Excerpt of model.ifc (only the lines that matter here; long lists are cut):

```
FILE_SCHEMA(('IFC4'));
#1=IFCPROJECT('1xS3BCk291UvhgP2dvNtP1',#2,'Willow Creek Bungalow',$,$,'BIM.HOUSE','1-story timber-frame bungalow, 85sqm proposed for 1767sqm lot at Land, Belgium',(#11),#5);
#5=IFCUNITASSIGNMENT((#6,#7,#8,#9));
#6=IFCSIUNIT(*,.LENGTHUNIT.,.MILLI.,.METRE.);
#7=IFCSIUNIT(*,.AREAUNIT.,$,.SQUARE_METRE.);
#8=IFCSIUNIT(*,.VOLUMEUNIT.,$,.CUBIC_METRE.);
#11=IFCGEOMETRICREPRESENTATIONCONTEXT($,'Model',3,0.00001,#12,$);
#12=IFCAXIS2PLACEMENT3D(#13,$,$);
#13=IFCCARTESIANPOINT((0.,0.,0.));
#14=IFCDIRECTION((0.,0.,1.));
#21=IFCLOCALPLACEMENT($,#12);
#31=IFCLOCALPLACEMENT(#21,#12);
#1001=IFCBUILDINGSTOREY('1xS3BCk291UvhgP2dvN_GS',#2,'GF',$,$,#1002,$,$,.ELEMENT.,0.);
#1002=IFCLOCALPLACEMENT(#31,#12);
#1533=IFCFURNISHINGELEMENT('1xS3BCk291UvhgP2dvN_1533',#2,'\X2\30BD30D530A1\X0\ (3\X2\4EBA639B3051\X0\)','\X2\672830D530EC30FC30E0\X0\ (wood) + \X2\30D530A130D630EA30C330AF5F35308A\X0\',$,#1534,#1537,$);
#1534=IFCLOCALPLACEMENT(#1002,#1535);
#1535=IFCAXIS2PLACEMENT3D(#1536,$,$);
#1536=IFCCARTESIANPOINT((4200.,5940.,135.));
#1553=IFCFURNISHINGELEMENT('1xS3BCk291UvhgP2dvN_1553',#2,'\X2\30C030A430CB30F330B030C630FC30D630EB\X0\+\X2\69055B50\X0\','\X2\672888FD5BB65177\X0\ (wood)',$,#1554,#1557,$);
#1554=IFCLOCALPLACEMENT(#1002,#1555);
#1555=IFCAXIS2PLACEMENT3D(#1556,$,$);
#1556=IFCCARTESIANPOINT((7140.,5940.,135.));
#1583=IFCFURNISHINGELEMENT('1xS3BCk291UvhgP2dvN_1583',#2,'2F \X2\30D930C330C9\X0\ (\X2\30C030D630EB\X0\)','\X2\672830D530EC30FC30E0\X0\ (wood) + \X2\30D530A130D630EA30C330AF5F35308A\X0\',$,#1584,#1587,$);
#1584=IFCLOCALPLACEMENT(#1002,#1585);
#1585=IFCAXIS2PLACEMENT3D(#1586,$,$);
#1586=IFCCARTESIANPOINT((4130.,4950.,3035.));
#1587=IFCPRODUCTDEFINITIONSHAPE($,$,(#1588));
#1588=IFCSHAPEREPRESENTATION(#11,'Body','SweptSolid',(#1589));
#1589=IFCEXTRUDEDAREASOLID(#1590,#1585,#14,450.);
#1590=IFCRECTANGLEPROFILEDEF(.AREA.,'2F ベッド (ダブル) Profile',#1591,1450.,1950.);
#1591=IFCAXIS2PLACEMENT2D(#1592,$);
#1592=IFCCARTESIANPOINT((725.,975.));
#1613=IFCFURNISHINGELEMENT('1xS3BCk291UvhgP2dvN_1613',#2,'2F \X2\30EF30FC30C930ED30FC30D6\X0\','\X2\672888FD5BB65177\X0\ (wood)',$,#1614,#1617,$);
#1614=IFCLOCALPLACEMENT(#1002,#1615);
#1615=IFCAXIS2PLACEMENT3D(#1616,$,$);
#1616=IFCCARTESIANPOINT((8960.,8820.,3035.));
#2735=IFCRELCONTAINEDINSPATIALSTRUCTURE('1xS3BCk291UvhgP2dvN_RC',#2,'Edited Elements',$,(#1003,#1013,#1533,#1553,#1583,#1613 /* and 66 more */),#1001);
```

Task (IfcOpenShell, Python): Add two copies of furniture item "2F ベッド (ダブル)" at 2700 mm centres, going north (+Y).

```python
import numpy as np
import ifcopenshell
import ifcopenshell.api.geometry
import ifcopenshell.api.root
import ifcopenshell.util.element
import ifcopenshell.util.placement

model = ifcopenshell.open("model.ifc")


def reuse_history(source, copy):
    """copy_class also copies each property set's owner history, people and application; keep the originals."""
    for rel in copy.IsDefinedBy:
        if rel.is_a("IfcRelDefinesByProperties") and (history := rel.RelatingPropertyDefinition.OwnerHistory):
            rel.RelatingPropertyDefinition.OwnerHistory = source.OwnerHistory
            ifcopenshell.util.element.remove_deep2(model, history)


source = model.by_guid("1xS3BCk291UvhgP2dvN_1583")
base = ifcopenshell.util.placement.get_local_placement(source.ObjectPlacement)
step = np.array([0.0, 1.0, 0.0]) * 2700.0

for i in range(1, 3):
    copy = ifcopenshell.api.root.copy_class(model, product=source)
    copy.Representation = ifcopenshell.util.element.copy_deep(
        model, source.Representation, exclude=["IfcGeometricRepresentationContext", "IfcRepresentationMap"]
    )
    reuse_history(source, copy)
    matrix = base.copy()
    matrix[:3, 3] += i * step
    print("added at", matrix[:3, 3].round(3) + 0.0)
    ifcopenshell.api.geometry.edit_object_placement(model, product=copy, matrix=matrix, is_si=False)

model.write("model_updated.ifc")
```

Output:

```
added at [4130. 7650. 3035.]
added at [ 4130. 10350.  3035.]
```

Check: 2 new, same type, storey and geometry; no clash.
